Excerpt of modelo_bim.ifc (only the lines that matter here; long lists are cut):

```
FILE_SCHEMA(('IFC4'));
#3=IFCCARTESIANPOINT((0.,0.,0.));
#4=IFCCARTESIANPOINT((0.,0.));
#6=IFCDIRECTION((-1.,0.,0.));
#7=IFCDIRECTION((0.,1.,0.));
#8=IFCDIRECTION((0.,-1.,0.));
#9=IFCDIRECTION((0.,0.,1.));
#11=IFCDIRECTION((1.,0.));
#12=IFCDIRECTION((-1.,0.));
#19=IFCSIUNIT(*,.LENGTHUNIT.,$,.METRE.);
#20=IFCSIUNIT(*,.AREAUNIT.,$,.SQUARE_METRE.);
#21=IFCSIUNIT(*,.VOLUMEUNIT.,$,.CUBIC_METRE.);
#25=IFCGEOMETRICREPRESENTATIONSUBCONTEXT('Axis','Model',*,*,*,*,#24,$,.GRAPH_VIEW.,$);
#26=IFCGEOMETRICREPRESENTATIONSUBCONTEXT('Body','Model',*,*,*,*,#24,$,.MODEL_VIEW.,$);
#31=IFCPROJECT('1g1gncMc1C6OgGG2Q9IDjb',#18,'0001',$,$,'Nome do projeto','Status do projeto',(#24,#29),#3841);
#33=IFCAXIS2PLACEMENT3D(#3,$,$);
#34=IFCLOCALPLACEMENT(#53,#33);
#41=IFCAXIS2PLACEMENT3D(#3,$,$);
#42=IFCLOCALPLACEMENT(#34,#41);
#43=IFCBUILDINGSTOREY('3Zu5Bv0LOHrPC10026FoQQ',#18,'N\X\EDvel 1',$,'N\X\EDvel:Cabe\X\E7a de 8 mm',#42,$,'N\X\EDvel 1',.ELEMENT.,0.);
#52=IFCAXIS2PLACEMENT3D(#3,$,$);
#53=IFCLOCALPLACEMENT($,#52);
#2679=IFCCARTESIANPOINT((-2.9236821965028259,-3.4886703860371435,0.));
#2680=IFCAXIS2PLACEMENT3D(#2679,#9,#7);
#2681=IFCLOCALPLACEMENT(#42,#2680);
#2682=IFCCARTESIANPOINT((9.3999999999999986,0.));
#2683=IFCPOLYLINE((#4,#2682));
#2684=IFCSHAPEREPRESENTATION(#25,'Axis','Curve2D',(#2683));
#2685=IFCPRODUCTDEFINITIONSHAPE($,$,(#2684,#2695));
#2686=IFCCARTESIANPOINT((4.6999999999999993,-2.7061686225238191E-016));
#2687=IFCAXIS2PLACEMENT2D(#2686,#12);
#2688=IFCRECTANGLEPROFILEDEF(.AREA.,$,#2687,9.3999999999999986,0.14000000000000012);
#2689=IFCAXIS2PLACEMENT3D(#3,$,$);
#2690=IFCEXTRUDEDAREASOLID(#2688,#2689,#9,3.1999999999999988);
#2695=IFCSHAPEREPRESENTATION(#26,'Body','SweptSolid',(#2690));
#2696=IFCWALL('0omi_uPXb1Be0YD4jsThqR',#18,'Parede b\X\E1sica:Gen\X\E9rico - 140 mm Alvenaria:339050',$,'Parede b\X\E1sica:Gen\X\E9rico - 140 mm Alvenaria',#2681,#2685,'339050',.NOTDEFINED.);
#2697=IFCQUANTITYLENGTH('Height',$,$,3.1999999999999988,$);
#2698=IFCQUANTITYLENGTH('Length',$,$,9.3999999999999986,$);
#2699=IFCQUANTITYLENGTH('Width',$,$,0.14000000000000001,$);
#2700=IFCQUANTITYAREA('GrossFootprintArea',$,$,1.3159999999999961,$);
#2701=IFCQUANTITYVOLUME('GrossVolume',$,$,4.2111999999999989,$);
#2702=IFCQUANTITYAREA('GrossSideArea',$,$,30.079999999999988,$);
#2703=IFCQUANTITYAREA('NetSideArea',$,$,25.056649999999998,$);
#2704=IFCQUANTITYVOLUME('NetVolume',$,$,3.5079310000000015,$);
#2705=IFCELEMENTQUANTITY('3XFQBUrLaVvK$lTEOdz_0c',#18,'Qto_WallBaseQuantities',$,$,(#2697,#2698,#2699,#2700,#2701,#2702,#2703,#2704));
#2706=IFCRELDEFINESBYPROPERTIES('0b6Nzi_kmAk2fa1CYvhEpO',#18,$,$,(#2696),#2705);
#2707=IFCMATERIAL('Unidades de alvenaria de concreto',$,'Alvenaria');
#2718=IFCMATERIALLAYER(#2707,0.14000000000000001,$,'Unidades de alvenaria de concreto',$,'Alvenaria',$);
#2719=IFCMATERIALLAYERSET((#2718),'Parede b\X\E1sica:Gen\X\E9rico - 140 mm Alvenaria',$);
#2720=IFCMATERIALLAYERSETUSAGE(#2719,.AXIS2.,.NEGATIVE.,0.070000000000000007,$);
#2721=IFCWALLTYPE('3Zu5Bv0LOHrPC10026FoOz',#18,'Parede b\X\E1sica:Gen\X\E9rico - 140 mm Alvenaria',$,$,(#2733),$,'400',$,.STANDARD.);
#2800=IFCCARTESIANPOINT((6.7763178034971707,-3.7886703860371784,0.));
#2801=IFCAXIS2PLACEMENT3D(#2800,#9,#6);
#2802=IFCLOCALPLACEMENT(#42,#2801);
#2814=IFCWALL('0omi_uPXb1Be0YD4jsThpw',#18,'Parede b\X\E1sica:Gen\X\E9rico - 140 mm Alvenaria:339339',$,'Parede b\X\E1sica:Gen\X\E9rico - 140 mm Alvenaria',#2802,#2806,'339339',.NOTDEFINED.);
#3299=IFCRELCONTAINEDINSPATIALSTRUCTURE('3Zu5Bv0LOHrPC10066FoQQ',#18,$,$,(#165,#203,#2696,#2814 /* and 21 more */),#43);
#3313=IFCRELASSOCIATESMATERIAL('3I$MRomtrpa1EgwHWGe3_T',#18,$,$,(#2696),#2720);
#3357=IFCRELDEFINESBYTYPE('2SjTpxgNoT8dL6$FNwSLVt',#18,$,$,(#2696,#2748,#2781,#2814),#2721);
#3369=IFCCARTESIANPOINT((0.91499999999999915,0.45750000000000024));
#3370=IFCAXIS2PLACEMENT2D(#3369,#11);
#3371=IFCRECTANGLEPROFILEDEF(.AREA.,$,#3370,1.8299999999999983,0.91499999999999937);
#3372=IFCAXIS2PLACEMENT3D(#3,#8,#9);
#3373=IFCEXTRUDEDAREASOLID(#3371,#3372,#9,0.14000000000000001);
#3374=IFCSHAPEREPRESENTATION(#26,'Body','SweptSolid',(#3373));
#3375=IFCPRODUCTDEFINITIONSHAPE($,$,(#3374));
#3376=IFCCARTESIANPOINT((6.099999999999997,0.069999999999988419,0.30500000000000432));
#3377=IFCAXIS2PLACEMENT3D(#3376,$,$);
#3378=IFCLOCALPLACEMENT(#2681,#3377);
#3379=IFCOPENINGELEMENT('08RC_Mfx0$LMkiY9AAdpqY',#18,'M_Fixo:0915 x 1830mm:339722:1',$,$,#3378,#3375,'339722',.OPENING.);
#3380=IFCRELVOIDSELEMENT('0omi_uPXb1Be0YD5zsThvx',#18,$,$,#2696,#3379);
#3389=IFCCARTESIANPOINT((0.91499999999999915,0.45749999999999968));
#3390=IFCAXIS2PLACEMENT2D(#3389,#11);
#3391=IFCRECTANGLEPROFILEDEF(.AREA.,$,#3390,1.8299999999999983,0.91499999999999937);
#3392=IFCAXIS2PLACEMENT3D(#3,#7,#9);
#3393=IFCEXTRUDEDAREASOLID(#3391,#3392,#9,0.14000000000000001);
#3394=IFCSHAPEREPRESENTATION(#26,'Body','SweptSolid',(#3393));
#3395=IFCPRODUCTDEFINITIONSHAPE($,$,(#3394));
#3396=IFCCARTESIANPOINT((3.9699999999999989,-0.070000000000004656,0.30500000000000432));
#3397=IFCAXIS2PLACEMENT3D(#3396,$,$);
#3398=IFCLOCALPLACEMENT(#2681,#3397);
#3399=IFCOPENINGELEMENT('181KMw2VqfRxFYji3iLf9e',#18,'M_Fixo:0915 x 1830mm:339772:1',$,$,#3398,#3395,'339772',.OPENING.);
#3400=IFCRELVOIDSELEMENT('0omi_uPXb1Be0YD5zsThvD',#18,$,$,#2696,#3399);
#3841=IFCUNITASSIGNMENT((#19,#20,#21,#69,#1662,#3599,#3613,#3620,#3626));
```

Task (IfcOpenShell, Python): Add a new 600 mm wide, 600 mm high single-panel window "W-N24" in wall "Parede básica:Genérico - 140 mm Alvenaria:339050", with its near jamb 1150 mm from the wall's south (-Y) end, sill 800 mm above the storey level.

```python
import numpy as np
import ifcopenshell
import ifcopenshell.api.feature
import ifcopenshell.api.geometry
import ifcopenshell.api.pset
import ifcopenshell.api.root
import ifcopenshell.api.spatial
import ifcopenshell.geom
import ifcopenshell.util.element
import ifcopenshell.util.placement
import ifcopenshell.util.representation
import ifcopenshell.util.shape
import ifcopenshell.util.unit

model = ifcopenshell.open("modelo_bim.ifc")
unit_scale = ifcopenshell.util.unit.calculate_unit_scale(model)
area_scale = ifcopenshell.util.unit.calculate_unit_scale(model, "AREAUNIT")
volume_scale = ifcopenshell.util.unit.calculate_unit_scale(model, "VOLUMEUNIT")
settings = ifcopenshell.geom.settings()


def volume(element):
    """Net volume in cubic metres, openings subtracted."""
    shape = ifcopenshell.geom.create_shape(settings, element)
    return ifcopenshell.util.shape.get_volume(shape.geometry)


wall = model.by_id(2696)
storey = ifcopenshell.util.element.get_container(wall, ifc_class="IfcBuildingStorey")
context = ifcopenshell.util.representation.get_context(model, "Model", "Body", "MODEL_VIEW")
before = volume(wall)

width, height, from_end, sill = 0.6, 0.6, 1.15, 0.8  # metres

# The wall runs along its own X axis, and the end named is its -X end.
wall_shape = ifcopenshell.geom.create_shape(settings, wall)
x, y, z = ifcopenshell.util.shape.get_vertices(wall_shape.geometry).T
start = x.min() + from_end
face, thickness = float(y.min()), float(y.max() - y.min())
wall_matrix = ifcopenshell.util.placement.get_local_placement(wall.ObjectPlacement)
level = ifcopenshell.util.placement.get_local_placement(storey.ObjectPlacement)[2, 3]


def in_wall(x, y):
    """Placement at x, y metres in the wall's axes, at sill height."""
    matrix = wall_matrix.copy()
    matrix[:, 3] = wall_matrix @ np.array([x / unit_scale, y / unit_scale, 0.0, 1.0])
    matrix[2, 3] = level + sill / unit_scale
    return matrix


# Opening: a box that overshoots both wall faces by 50 mm.
opening = ifcopenshell.api.root.create_entity(model, ifc_class="IfcOpeningElement", predefined_type="OPENING")
box = ifcopenshell.api.geometry.add_wall_representation(
    model, context=context, length=width, height=height, thickness=thickness + 0.1
)
ifcopenshell.api.geometry.assign_representation(model, product=opening, representation=box)
ifcopenshell.api.geometry.edit_object_placement(model, product=opening, matrix=in_wall(start, face - 0.05), is_si=False)
ifcopenshell.api.feature.add_feature(model, feature=opening, element=wall)

window = ifcopenshell.api.root.create_entity(model, ifc_class="IfcWindow", name="W-N24", predefined_type="WINDOW")
window.OverallWidth, window.OverallHeight = width / unit_scale, height / unit_scale
window.PartitioningType = "SINGLE_PANEL"
body = ifcopenshell.api.geometry.add_window_representation(
    model,
    context=context,
    overall_width=window.OverallWidth,
    overall_height=window.OverallHeight,
    partition_type="SINGLE_PANEL",
)
ifcopenshell.api.geometry.assign_representation(model, product=window, representation=body)
ifcopenshell.api.spatial.assign_container(model, products=[window], relating_structure=storey)
ifcopenshell.api.feature.add_filling(model, opening=opening, element=window)

# Centre the window in the wall's thickness.
ifcopenshell.api.geometry.edit_object_placement(model, product=window, matrix=in_wall(start, face), is_si=False)
window_shape = ifcopenshell.geom.create_shape(settings, window)
depth = ifcopenshell.util.shape.get_vertices(window_shape.geometry)[:, 1]
offset = face + thickness / 2 - (depth.min() + depth.max()) / 2
ifcopenshell.api.geometry.edit_object_placement(model, product=window, matrix=in_wall(start, offset), is_si=False)

after = volume(wall)

# Update the wall's stored quantities.
qto = model.by_id(ifcopenshell.util.element.get_pset(wall, "Qto_WallBaseQuantities", should_inherit=False)["id"])
ifcopenshell.api.pset.edit_qto(model, qto=qto, properties={
    "NetSideArea": after / thickness / area_scale,
    "NetVolume": after / volume_scale,
})

print(f"wall volume {before:.3f} -> {after:.3f} m3")

model.write("modelo_bim-out.ifc")
```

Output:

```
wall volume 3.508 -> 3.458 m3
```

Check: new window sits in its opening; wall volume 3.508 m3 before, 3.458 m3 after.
